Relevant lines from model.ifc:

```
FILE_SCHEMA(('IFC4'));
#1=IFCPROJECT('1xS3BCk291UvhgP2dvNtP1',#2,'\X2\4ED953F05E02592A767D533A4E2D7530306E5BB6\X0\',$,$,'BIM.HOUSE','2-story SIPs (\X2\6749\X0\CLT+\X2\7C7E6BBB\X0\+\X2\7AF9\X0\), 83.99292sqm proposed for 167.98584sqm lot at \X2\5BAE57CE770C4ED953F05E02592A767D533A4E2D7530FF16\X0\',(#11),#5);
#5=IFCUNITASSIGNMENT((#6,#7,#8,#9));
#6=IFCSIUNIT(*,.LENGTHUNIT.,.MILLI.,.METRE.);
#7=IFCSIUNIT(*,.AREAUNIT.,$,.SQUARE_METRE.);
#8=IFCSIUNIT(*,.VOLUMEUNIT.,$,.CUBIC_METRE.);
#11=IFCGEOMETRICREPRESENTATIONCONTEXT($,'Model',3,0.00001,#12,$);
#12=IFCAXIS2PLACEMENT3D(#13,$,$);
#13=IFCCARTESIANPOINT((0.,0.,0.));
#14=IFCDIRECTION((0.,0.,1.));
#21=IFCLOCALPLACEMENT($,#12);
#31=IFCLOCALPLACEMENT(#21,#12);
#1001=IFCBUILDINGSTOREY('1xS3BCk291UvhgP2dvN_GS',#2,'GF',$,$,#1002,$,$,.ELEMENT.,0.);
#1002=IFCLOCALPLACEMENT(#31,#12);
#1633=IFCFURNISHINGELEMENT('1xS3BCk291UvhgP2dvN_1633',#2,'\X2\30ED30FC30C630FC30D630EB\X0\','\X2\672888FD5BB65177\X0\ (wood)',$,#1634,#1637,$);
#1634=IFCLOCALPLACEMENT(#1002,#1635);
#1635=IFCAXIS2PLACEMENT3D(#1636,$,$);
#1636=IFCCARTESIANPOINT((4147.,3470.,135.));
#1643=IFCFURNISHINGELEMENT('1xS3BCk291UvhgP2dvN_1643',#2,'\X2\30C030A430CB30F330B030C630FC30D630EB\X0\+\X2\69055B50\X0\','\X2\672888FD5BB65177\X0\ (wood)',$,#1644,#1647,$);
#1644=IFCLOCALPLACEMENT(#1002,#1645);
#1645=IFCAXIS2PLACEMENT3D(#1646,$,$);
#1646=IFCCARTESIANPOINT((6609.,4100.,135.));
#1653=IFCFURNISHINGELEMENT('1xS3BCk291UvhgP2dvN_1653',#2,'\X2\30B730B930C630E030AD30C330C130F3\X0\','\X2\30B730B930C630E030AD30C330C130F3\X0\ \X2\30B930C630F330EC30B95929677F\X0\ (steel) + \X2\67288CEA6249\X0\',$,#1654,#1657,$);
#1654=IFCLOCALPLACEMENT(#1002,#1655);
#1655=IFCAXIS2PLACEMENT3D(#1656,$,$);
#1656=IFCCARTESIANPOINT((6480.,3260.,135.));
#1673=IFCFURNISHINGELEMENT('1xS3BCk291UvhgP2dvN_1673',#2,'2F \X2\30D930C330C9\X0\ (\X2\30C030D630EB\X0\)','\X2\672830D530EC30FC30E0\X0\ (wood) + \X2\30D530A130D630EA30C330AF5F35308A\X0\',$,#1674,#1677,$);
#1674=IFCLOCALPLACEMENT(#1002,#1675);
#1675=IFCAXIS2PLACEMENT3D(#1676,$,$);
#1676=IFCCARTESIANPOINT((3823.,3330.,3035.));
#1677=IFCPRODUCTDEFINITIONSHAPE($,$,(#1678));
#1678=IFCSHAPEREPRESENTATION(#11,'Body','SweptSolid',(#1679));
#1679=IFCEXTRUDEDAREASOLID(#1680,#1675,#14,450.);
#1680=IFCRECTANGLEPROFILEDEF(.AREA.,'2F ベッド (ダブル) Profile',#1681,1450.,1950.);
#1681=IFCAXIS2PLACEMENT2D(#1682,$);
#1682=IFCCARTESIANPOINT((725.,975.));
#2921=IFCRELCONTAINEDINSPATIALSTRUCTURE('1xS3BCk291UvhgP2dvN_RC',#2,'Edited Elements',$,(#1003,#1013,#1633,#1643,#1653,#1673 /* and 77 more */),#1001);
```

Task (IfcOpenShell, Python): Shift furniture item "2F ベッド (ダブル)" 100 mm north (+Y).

```python
import ifcopenshell
import ifcopenshell.api.geometry
import ifcopenshell.util.placement

model = ifcopenshell.open("model.ifc")

item = model.by_guid("1xS3BCk291UvhgP2dvN_1673")
matrix = ifcopenshell.util.placement.get_local_placement(item.ObjectPlacement)
matrix[1, 3] += 100.0
ifcopenshell.api.geometry.edit_object_placement(model, product=item, matrix=matrix, is_si=False)

print(ifcopenshell.util.placement.get_local_placement(item.ObjectPlacement).round(3) + 0.0)

model.write("model_updated.ifc")
```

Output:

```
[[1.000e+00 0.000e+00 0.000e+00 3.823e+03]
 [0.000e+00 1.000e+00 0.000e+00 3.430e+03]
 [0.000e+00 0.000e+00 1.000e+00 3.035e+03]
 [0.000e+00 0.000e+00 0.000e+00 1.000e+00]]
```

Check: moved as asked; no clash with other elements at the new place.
